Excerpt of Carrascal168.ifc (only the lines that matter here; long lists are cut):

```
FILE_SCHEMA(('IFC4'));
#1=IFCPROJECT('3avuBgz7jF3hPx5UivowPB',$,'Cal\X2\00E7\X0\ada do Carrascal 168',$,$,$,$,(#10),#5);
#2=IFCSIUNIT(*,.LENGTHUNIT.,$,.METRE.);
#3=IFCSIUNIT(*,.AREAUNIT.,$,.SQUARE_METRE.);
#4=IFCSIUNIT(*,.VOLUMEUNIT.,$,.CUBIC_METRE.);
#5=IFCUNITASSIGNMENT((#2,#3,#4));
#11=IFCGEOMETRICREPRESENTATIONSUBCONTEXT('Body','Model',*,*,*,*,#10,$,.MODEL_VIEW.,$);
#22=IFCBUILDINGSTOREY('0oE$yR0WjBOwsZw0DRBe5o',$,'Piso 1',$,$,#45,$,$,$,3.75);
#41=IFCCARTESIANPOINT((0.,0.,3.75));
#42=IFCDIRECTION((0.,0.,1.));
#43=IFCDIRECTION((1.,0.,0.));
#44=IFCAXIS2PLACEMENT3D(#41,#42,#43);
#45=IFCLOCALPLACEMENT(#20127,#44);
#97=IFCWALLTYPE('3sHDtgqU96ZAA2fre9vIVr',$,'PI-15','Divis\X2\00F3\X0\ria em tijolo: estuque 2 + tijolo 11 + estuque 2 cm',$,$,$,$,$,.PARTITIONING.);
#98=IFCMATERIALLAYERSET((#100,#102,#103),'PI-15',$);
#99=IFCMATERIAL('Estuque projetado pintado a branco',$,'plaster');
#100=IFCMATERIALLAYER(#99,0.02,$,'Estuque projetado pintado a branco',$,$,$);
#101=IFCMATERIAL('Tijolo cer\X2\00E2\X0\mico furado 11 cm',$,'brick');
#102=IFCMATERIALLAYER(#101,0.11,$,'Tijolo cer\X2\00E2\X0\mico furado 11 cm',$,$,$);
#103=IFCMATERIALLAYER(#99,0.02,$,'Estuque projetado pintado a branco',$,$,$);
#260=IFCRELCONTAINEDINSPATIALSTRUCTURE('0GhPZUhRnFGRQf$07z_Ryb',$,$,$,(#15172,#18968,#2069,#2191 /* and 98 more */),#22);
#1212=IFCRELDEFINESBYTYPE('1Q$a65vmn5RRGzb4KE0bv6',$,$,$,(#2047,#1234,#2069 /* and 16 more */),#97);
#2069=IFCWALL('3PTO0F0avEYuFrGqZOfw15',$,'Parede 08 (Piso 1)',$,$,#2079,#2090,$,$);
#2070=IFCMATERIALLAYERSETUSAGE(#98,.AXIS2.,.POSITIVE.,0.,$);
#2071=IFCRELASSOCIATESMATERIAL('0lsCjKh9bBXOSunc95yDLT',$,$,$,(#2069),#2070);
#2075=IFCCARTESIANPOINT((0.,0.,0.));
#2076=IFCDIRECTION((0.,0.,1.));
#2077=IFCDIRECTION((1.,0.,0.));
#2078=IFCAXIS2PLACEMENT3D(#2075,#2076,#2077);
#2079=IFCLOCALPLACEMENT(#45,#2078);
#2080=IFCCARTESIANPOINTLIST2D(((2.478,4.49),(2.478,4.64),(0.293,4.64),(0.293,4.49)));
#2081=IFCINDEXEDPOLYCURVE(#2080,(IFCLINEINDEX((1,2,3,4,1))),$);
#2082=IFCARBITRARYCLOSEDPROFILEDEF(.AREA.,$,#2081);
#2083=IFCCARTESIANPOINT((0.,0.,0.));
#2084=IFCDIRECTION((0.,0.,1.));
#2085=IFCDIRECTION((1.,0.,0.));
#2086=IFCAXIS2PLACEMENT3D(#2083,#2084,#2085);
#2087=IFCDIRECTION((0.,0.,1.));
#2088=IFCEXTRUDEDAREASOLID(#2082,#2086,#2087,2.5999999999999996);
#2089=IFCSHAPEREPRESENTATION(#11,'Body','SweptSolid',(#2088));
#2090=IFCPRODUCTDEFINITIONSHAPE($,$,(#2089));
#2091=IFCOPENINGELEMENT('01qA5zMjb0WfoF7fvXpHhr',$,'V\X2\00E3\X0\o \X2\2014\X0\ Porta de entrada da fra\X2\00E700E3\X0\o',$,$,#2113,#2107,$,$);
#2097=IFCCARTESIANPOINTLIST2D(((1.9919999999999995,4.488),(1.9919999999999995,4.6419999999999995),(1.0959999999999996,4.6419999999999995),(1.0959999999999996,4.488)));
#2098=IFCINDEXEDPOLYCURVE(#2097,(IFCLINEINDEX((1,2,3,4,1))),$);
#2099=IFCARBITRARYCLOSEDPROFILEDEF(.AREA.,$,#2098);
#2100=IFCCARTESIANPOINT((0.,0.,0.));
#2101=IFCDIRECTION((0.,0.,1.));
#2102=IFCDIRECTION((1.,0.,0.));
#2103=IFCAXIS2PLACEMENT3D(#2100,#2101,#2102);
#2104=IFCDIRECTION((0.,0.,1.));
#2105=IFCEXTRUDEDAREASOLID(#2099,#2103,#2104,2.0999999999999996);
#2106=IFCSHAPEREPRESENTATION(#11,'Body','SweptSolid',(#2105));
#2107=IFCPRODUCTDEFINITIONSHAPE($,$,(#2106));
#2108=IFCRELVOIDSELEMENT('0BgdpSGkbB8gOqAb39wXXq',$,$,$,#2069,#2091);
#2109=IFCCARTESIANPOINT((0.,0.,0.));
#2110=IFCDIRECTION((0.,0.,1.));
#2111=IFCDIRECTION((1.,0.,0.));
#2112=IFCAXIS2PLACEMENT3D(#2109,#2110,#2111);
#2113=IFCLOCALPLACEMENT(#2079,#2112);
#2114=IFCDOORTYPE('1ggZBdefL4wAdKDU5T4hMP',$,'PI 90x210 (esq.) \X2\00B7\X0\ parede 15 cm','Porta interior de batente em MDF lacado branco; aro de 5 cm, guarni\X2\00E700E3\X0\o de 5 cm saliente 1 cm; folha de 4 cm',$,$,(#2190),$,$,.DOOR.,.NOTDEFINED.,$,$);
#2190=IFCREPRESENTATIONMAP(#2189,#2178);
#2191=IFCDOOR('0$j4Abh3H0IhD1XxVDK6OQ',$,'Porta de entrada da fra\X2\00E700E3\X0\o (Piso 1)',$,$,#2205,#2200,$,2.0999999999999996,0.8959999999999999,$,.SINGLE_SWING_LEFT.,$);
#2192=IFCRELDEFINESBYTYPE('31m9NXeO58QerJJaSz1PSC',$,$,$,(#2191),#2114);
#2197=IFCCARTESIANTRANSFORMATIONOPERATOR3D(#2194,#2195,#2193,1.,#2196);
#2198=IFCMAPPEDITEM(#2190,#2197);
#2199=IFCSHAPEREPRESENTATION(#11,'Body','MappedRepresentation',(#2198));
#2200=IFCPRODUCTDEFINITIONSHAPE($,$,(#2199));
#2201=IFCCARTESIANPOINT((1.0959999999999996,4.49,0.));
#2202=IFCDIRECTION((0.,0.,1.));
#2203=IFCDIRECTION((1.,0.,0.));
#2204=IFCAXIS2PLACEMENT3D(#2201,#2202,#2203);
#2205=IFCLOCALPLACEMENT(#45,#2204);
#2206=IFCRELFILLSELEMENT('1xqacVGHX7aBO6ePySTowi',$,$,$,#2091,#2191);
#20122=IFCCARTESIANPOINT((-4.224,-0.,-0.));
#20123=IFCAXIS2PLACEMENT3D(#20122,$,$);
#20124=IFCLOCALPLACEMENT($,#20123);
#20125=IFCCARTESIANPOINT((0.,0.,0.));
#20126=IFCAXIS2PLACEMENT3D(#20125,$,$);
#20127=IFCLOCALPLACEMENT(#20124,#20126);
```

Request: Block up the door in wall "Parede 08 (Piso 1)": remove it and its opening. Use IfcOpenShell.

```python
import ifcopenshell
import ifcopenshell.api.feature
import ifcopenshell.api.root
import ifcopenshell.geom
import ifcopenshell.util.shape

model = ifcopenshell.open("Carrascal168.ifc")
settings = ifcopenshell.geom.settings()


def volume(element):
    """Net volume in cubic metres, openings subtracted."""
    shape = ifcopenshell.geom.create_shape(settings, element)
    return ifcopenshell.util.shape.get_volume(shape.geometry)


door = model.by_guid("0$j4Abh3H0IhD1XxVDK6OQ")
opening = door.FillsVoids[0].RelatingOpeningElement
wall = opening.VoidsElements[0].RelatingBuildingElement
before = volume(wall)

ifcopenshell.api.root.remove_product(model, product=door)
ifcopenshell.api.feature.remove_feature(model, feature=opening)

after = volume(wall)

print(f"wall volume {before:.3f} -> {after:.3f} m3")

model.write("Carrascal168-out.ifc")
```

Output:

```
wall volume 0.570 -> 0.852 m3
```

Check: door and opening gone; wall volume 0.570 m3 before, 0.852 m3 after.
